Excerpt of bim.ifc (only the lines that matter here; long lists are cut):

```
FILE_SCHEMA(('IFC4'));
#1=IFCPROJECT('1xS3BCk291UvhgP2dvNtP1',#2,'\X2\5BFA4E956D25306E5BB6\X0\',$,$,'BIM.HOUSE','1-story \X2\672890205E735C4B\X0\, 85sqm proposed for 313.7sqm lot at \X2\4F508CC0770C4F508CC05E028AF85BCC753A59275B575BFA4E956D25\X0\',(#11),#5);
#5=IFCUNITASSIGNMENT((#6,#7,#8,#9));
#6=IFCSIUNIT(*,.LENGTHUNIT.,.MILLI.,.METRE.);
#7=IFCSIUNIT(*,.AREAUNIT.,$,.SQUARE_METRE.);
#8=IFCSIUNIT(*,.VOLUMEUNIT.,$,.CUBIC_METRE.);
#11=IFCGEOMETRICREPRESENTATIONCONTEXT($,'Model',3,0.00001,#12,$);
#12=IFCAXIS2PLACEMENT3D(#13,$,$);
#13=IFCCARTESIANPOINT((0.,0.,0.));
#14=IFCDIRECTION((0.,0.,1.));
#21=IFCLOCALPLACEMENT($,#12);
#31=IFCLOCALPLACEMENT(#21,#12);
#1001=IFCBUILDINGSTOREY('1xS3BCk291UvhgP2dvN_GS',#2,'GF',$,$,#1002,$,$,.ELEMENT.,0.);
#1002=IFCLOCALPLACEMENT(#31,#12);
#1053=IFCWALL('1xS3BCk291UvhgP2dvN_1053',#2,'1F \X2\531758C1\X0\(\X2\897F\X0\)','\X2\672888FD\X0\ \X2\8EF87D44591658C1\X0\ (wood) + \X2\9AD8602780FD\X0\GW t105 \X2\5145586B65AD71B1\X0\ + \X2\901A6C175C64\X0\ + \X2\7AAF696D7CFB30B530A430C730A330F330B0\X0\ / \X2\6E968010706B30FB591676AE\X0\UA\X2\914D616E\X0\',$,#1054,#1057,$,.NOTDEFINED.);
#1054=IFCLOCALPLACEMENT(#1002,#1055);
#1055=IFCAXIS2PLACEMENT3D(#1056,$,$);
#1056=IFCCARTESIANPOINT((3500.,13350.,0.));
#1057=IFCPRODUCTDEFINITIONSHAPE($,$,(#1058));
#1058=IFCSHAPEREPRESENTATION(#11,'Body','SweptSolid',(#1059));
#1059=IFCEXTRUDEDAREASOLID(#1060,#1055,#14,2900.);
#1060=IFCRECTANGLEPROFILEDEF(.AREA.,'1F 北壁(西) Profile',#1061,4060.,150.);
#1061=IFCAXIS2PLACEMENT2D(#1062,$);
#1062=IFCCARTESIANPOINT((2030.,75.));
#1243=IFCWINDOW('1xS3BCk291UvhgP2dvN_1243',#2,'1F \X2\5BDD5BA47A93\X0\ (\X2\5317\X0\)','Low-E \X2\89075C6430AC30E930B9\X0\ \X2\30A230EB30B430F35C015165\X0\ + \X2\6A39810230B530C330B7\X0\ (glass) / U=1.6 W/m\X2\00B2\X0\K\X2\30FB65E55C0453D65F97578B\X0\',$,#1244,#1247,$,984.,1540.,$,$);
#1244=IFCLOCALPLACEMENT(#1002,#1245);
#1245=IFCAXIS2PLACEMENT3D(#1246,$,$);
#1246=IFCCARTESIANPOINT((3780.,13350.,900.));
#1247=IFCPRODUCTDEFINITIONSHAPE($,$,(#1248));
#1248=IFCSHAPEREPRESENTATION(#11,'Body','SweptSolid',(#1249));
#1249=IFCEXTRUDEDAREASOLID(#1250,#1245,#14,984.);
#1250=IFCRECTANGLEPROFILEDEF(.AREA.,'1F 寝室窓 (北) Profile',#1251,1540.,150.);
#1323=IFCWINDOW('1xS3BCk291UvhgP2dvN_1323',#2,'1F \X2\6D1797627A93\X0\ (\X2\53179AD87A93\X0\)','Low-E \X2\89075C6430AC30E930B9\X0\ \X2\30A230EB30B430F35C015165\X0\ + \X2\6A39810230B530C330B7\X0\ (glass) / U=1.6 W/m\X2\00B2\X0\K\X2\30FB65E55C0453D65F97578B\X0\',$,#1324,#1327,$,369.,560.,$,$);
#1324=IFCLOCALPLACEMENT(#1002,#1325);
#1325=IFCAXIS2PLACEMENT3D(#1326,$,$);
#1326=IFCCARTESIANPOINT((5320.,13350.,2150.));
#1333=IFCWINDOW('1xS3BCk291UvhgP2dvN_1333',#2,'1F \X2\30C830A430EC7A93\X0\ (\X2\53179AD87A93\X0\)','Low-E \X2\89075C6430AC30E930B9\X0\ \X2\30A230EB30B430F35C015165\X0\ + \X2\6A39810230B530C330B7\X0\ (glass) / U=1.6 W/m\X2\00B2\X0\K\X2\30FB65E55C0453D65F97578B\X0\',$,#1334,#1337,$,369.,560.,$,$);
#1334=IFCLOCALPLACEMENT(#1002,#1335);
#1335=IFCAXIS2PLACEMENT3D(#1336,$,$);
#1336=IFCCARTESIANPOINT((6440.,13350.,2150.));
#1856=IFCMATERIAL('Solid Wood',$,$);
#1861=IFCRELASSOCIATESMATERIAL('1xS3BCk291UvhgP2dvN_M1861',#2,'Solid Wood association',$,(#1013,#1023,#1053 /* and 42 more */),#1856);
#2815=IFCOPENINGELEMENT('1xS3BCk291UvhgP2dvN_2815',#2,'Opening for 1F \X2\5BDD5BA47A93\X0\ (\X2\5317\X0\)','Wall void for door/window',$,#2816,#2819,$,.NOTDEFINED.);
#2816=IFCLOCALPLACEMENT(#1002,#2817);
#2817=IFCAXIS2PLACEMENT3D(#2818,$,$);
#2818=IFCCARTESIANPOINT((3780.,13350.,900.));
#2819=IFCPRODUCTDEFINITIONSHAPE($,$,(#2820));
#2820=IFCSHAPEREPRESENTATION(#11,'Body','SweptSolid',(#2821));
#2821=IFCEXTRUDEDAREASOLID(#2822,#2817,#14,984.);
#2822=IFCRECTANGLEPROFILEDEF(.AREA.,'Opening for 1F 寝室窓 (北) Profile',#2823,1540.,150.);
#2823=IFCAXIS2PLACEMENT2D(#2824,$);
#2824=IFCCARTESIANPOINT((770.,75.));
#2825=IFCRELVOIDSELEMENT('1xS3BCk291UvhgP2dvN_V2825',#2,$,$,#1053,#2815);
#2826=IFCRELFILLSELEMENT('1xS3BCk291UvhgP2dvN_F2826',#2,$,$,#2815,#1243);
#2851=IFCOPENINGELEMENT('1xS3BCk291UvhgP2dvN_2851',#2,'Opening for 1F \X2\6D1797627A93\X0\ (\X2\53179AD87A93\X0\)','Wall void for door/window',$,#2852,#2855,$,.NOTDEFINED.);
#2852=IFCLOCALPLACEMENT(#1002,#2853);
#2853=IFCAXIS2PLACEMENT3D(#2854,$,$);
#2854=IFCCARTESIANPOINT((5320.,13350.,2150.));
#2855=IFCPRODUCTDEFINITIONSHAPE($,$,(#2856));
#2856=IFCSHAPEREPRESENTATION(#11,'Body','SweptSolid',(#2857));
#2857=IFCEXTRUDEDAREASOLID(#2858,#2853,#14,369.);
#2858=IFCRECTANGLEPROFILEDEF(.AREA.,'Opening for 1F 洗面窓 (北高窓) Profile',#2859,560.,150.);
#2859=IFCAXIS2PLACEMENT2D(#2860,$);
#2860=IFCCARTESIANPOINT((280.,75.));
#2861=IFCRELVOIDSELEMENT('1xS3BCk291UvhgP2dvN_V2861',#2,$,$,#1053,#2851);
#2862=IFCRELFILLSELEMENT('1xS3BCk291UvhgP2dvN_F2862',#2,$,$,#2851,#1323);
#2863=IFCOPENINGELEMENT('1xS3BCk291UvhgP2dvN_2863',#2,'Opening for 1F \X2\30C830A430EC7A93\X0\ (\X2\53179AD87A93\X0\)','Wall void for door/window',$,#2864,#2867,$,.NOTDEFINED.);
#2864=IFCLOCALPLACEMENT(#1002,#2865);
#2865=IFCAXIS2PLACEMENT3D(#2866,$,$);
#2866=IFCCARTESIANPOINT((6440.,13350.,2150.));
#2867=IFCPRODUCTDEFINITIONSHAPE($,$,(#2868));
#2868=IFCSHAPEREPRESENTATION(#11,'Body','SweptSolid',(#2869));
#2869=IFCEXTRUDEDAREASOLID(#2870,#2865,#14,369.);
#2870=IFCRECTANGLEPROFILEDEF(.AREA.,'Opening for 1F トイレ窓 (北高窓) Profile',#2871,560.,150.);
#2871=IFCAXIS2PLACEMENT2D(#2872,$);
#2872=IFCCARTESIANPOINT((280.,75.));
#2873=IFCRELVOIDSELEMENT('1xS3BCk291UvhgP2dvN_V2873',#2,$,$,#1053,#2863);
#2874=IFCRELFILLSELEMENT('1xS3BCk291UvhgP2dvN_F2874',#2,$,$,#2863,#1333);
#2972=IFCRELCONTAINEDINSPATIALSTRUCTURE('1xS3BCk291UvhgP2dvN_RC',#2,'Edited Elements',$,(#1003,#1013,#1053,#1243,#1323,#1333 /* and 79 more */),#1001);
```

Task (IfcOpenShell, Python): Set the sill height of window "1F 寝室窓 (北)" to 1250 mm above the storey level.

```python
import numpy as np
import ifcopenshell
import ifcopenshell.api.geometry
import ifcopenshell.geom
import ifcopenshell.util.element
import ifcopenshell.util.placement
import ifcopenshell.util.shape
import ifcopenshell.util.unit

model = ifcopenshell.open("bim.ifc")
unit_scale = ifcopenshell.util.unit.calculate_unit_scale(model)

window = model.by_guid("1xS3BCk291UvhgP2dvN_1243")
opening = window.FillsVoids[0].RelatingOpeningElement
storey = ifcopenshell.util.element.get_container(window, ifc_class="IfcBuildingStorey")
level = ifcopenshell.util.placement.get_local_placement(storey.ObjectPlacement)[2, 3]

# The opening's origin need not be at the sill, so measure its lowest point.
shape = ifcopenshell.geom.create_shape(ifcopenshell.geom.settings(), opening)
bottom = ifcopenshell.util.shape.get_shape_bottom_elevation(shape, shape.geometry) / unit_scale
dz = level + 1.25 / unit_scale - bottom

shift = np.array([0.0, 0.0, dz])
# The window is not placed relative to its opening, so move both.
for product in (opening, window):
    matrix = ifcopenshell.util.placement.get_local_placement(product.ObjectPlacement)
    matrix[:3, 3] += shift
    ifcopenshell.api.geometry.edit_object_placement(model, product=product, matrix=matrix, is_si=False)

print(f"moved by {dz * unit_scale:+.3f} m")

model.write("bim_edited.ifc")
```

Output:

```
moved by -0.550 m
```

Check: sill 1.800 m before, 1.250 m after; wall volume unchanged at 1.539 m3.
